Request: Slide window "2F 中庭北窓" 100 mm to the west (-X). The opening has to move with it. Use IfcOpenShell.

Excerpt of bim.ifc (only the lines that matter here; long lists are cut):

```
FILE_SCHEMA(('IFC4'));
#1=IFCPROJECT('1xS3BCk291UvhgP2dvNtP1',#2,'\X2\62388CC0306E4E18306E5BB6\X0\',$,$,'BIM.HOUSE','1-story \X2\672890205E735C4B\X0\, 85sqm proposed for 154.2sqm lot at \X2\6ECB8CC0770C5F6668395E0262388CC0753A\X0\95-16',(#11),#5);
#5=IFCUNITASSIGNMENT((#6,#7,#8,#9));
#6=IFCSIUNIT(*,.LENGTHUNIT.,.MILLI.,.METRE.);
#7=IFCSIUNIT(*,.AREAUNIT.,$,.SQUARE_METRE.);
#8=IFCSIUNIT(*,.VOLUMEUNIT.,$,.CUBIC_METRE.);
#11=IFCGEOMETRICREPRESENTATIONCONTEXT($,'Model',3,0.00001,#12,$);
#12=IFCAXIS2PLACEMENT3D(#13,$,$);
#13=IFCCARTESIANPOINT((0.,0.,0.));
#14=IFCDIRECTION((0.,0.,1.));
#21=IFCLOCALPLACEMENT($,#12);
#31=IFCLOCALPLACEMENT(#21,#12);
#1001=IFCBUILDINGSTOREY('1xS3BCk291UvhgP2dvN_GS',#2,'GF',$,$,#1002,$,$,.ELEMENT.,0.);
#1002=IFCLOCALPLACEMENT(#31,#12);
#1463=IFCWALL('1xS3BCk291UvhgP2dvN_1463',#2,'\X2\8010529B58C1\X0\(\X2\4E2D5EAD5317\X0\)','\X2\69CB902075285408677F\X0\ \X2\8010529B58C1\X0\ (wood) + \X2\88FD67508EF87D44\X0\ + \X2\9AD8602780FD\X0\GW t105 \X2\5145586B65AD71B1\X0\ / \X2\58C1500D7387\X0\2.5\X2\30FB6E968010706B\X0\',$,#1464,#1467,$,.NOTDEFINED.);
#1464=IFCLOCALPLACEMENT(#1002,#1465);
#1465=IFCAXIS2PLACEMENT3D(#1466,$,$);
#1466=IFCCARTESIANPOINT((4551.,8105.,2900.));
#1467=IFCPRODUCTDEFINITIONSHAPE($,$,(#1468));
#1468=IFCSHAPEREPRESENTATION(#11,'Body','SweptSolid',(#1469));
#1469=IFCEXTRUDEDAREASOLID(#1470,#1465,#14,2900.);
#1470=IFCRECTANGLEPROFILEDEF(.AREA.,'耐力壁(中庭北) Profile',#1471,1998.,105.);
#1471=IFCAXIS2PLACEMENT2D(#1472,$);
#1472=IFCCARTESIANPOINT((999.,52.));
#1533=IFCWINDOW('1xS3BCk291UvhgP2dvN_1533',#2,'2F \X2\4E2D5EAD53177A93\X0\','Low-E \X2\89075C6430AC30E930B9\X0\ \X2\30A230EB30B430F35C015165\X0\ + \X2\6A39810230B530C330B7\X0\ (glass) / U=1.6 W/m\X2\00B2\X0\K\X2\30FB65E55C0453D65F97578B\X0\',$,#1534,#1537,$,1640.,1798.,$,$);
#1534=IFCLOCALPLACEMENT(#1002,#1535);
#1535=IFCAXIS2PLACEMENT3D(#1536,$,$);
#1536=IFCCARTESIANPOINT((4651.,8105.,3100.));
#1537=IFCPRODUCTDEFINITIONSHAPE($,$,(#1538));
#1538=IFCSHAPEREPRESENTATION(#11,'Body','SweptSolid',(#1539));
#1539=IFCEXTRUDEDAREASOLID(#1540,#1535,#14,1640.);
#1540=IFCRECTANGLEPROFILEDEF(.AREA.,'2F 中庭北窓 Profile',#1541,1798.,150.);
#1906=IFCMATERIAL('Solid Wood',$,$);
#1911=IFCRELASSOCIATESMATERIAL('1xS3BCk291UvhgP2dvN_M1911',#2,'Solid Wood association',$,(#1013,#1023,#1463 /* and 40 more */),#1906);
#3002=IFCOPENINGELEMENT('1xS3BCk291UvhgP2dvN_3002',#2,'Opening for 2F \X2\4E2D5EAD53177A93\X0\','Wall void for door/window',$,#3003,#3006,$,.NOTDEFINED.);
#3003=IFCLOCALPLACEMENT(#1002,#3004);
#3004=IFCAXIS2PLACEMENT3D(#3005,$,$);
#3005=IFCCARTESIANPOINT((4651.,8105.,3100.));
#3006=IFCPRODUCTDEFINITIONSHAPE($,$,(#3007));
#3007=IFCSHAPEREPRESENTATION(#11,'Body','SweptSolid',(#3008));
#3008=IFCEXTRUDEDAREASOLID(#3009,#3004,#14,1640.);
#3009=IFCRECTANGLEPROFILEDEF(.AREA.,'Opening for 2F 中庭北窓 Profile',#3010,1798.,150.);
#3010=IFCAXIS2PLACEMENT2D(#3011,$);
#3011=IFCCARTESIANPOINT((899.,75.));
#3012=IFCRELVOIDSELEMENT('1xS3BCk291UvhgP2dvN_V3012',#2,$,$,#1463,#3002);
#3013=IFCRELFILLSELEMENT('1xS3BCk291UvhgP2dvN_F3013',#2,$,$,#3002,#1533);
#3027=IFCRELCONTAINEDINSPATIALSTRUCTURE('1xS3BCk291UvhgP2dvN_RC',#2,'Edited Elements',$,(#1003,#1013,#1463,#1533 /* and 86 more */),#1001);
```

```python
import ifcopenshell
import ifcopenshell.api.geometry
import ifcopenshell.util.placement

model = ifcopenshell.open("bim.ifc")

window = model.by_guid("1xS3BCk291UvhgP2dvN_1533")
opening = window.FillsVoids[0].RelatingOpeningElement
wall = opening.VoidsElements[0].RelatingBuildingElement

wall_matrix = ifcopenshell.util.placement.get_local_placement(wall.ObjectPlacement)
shift = wall_matrix[:3, 0] * -100.0
before = ifcopenshell.util.placement.get_local_placement(window.ObjectPlacement)[:3, 3].copy()

# The window is not placed relative to its opening, so move both.
for product in (opening, window):
    matrix = ifcopenshell.util.placement.get_local_placement(product.ObjectPlacement)
    matrix[:3, 3] += shift
    ifcopenshell.api.geometry.edit_object_placement(model, product=product, matrix=matrix, is_si=False)

after = ifcopenshell.util.placement.get_local_placement(window.ObjectPlacement)[:3, 3]
print("window moved by", (after - before).round(3) + 0.0)

model.write("bim_rev.ifc")
```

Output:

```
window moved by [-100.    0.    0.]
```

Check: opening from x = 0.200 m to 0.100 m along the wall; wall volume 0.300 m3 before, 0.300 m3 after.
